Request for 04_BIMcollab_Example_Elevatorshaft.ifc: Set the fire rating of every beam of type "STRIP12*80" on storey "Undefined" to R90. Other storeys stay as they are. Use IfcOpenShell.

First a look at what the model holds.

```python
import ifcopenshell
import ifcopenshell.util.element

model = ifcopenshell.open("04_BIMcollab_Example_Elevatorshaft.ifc")
print(model.schema)
storey = next(s for s in model.by_type("IfcBuildingStorey") if s.Name == "Undefined")
beams = [e for e in ifcopenshell.util.element.get_decomposition(storey) if e.is_a("IfcBeam")]
seen = {}
for e in beams:
    element_type = ifcopenshell.util.element.get_type(e)
    key = (element_type.Name if element_type != e and element_type else None, ifcopenshell.util.element.get_pset(e, "Pset_BeamCommon", "FireRating"))
    seen[key] = seen.get(key, 0) + 1
for (name, value), count in sorted(seen.items(), key=str):
    print(count, "x", name, "|", value)
```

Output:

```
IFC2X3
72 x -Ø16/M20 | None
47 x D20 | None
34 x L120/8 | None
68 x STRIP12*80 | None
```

```python
import ifcopenshell
import ifcopenshell.api.pset
import ifcopenshell.util.element

model = ifcopenshell.open("04_BIMcollab_Example_Elevatorshaft.ifc")

storey = next(s for s in model.by_type("IfcBuildingStorey") if s.Name == "Undefined")
beams = [e for e in ifcopenshell.util.element.get_decomposition(storey) if e.is_a("IfcBeam")]

count = 0
for e in beams:
    element_type = ifcopenshell.util.element.get_type(e)
    if element_type in (None, e) or element_type.Name != "STRIP12*80":
        continue
    # add_pset returns the element's existing set when there is one.
    pset = ifcopenshell.api.pset.add_pset(model, product=e, name="Pset_BeamCommon")
    ifcopenshell.api.pset.edit_pset(model, pset=pset, properties={"FireRating": "R90"})
    count += 1

print(count, "beams updated")

model.write("04_BIMcollab_Example_Elevatorshaft_v2.ifc")
```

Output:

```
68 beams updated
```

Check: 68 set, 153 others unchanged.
